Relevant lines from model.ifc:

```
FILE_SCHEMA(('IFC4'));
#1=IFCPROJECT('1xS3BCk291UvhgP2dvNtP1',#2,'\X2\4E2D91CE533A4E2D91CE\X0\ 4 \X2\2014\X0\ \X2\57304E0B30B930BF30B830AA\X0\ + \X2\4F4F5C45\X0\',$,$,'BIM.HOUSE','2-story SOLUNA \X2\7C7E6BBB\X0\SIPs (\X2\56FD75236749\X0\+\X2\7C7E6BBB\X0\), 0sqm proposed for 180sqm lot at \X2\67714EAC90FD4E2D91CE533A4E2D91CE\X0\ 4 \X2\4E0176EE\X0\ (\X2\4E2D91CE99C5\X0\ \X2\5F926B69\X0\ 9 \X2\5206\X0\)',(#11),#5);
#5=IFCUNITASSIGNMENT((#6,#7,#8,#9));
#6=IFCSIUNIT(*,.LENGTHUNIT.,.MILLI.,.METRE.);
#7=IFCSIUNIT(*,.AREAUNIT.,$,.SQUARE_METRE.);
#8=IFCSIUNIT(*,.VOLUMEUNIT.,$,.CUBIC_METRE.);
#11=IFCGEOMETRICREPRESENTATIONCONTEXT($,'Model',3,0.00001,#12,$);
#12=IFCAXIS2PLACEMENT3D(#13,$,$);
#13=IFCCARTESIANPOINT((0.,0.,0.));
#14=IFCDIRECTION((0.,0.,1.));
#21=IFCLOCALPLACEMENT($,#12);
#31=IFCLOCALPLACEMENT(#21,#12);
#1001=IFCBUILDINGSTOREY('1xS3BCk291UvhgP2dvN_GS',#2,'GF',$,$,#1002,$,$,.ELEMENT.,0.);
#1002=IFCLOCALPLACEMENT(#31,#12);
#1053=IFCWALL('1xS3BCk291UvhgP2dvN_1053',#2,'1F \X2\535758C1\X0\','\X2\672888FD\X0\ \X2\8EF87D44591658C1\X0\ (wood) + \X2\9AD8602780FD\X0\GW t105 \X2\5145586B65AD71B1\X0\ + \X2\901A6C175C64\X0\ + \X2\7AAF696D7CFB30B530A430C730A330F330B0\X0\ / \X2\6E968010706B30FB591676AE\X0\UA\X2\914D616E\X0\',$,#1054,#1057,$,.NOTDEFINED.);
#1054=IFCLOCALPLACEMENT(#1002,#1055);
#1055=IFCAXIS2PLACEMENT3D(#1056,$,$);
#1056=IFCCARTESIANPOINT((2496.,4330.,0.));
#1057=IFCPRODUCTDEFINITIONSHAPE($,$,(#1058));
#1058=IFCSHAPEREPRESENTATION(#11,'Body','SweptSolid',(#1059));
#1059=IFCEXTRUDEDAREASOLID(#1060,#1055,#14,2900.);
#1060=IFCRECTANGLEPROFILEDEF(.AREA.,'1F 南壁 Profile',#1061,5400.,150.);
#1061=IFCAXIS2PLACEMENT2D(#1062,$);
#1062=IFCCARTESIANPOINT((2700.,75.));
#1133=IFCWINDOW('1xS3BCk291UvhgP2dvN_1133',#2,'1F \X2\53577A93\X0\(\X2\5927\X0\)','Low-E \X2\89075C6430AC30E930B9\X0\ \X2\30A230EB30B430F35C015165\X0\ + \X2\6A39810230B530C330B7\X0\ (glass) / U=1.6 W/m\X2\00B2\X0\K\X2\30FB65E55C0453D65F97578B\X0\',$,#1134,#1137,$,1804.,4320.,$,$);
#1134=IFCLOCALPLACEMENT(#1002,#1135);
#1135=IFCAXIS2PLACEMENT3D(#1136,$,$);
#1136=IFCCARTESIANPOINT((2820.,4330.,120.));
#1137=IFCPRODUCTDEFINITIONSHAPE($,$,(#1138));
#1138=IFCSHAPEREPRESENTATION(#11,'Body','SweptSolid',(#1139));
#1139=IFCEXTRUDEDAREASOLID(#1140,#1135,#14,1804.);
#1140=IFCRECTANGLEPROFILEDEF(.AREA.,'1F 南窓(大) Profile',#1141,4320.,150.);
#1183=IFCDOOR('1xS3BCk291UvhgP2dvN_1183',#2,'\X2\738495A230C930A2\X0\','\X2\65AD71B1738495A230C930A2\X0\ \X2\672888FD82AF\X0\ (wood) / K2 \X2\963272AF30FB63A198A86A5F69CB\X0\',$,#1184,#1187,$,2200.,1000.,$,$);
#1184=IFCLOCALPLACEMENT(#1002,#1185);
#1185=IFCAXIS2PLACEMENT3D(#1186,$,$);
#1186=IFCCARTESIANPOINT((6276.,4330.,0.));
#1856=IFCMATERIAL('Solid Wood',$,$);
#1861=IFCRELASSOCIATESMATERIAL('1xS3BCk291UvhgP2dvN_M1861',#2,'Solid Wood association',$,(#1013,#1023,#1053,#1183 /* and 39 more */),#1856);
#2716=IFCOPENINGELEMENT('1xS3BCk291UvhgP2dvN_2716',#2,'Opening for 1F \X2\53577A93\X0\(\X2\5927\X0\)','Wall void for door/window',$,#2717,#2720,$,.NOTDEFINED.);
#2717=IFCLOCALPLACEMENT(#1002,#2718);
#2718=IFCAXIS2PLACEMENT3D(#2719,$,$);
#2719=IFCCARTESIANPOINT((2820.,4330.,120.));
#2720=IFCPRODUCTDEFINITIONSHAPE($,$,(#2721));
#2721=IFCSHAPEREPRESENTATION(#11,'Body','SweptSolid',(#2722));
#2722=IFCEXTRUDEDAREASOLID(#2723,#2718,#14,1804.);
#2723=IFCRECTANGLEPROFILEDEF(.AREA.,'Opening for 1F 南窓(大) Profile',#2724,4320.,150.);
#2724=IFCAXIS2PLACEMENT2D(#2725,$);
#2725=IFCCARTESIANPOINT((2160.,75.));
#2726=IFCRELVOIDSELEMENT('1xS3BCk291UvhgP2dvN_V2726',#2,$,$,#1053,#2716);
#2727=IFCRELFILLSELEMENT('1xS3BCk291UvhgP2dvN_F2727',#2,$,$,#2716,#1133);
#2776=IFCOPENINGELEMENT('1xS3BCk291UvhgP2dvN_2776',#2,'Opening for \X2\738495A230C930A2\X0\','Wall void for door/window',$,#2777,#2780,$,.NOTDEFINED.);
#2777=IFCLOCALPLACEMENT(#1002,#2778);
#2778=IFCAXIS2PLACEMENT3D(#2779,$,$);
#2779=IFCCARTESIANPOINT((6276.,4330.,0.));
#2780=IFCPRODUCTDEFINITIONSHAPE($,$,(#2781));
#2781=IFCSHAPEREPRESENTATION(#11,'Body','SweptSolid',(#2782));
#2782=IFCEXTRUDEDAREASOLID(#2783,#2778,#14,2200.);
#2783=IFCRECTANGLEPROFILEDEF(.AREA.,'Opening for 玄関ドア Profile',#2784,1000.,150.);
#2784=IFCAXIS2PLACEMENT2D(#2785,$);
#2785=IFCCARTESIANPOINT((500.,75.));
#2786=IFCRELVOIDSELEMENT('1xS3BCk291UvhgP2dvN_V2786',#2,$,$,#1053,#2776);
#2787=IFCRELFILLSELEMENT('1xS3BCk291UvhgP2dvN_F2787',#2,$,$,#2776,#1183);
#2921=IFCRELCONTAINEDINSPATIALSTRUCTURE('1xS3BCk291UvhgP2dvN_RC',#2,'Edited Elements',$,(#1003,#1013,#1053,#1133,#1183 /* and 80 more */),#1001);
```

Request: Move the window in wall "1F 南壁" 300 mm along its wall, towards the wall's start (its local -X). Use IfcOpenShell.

```python
import ifcopenshell
import ifcopenshell.api.geometry
import ifcopenshell.util.placement

model = ifcopenshell.open("model.ifc")

window = model.by_guid("1xS3BCk291UvhgP2dvN_1133")
opening = window.FillsVoids[0].RelatingOpeningElement
wall = opening.VoidsElements[0].RelatingBuildingElement

wall_matrix = ifcopenshell.util.placement.get_local_placement(wall.ObjectPlacement)
shift = wall_matrix[:3, 0] * -300.0
before = ifcopenshell.util.placement.get_local_placement(window.ObjectPlacement)[:3, 3].copy()

# The window is not placed relative to its opening, so move both.
for product in (opening, window):
    matrix = ifcopenshell.util.placement.get_local_placement(product.ObjectPlacement)
    matrix[:3, 3] += shift
    ifcopenshell.api.geometry.edit_object_placement(model, product=product, matrix=matrix, is_si=False)

after = ifcopenshell.util.placement.get_local_placement(window.ObjectPlacement)[:3, 3]
print("window moved by", (after - before).round(3) + 0.0)

model.write("model_updated.ifc")
```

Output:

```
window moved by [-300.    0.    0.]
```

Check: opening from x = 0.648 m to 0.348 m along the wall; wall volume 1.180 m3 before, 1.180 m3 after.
